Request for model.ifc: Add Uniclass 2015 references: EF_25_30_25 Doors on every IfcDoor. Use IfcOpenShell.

First a look at what the model holds.

```python
import ifcopenshell

model = ifcopenshell.open("model.ifc")
print(model.schema)
print("classifications:", [c.Name for c in model.by_type("IfcClassification")])
for ifc_class in ("IfcDoor", "IfcRoof", "IfcStair", "IfcWall", "IfcWindow"):
    print(ifc_class, len(model.by_type(ifc_class)))
```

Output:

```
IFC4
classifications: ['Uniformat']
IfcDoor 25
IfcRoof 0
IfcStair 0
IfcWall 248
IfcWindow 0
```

```python
import ifcopenshell
import ifcopenshell.api.classification

model = ifcopenshell.open("model.ifc")

system = ifcopenshell.api.classification.add_classification(model, classification="Uniclass 2015")

codes = {
    "IfcDoor": ("EF_25_30_25", "Doors"),
}
for ifc_class, (code, name) in codes.items():
    products = model.by_type(ifc_class)
    ifcopenshell.api.classification.add_reference(
        model, products=products, classification=system, identification=code, name=name
    )
    print(code, len(products))

model.write("model-out.ifc")
```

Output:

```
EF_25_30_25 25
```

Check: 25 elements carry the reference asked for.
